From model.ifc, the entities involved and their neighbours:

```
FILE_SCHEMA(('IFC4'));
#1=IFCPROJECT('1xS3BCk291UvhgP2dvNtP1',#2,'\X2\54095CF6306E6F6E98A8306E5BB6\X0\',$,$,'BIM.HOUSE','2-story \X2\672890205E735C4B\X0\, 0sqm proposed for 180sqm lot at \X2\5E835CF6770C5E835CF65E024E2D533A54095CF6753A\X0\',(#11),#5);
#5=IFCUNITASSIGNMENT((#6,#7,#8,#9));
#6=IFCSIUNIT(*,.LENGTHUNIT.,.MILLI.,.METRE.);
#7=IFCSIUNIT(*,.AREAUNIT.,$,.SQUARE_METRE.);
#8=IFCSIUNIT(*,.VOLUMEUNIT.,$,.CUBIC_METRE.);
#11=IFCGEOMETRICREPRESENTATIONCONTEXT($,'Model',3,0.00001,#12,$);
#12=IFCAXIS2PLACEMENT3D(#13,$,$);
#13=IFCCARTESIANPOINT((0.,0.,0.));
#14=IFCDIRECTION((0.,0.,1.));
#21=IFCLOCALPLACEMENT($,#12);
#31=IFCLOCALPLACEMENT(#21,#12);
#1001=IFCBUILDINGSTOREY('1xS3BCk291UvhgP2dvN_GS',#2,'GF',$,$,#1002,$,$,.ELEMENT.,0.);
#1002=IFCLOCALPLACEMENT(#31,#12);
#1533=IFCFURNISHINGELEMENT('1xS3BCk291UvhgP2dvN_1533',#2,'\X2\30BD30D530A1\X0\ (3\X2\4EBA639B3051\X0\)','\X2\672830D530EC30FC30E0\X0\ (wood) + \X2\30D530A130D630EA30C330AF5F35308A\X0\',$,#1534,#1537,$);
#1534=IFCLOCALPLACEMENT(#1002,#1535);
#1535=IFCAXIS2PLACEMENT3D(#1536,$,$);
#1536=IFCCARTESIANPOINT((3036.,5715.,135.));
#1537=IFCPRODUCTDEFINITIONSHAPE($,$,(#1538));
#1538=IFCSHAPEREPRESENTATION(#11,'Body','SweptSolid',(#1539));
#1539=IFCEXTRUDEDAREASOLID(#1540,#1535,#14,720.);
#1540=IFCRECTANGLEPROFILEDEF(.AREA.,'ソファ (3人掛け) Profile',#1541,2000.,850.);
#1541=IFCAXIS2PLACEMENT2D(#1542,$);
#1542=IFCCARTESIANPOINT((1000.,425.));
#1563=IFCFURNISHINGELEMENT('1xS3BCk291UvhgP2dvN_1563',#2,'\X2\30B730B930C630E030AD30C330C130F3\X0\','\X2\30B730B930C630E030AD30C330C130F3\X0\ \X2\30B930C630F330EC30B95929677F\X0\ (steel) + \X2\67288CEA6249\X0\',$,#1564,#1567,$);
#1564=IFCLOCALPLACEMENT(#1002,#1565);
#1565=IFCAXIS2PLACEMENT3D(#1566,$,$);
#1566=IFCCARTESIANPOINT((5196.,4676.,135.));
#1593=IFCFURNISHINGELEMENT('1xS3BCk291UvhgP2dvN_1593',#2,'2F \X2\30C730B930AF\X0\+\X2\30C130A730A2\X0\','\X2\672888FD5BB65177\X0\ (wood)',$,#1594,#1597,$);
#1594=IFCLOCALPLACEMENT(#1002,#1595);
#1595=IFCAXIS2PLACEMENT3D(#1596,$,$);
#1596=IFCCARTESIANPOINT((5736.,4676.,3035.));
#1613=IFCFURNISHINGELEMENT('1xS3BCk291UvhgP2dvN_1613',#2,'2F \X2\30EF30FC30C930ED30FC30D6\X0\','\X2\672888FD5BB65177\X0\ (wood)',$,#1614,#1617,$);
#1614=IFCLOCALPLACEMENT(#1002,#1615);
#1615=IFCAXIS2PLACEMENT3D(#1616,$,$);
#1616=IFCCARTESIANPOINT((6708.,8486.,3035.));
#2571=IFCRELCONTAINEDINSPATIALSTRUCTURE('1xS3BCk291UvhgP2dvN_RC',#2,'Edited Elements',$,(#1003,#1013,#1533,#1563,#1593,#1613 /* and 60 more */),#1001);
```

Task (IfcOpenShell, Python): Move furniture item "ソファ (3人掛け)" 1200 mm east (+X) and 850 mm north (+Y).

```python
import ifcopenshell
import ifcopenshell.api.geometry
import ifcopenshell.util.placement

model = ifcopenshell.open("model.ifc")

item = model.by_guid("1xS3BCk291UvhgP2dvN_1533")
matrix = ifcopenshell.util.placement.get_local_placement(item.ObjectPlacement)
matrix[0, 3] += 1200.0
matrix[1, 3] += 850.0
ifcopenshell.api.geometry.edit_object_placement(model, product=item, matrix=matrix, is_si=False)

print(ifcopenshell.util.placement.get_local_placement(item.ObjectPlacement).round(3) + 0.0)

model.write("model_edited.ifc")
```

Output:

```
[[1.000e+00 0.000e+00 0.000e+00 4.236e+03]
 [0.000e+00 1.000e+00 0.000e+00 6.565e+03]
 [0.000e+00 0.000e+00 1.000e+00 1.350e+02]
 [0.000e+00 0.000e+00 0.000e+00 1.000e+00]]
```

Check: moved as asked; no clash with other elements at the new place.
